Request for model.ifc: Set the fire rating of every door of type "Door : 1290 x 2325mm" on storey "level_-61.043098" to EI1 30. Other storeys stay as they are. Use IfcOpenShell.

First a look at what the model holds.

```python
import ifcopenshell
import ifcopenshell.util.element

model = ifcopenshell.open("model.ifc")
print(model.schema)
storey = next(s for s in model.by_type("IfcBuildingStorey") if s.Name == "level_-61.043098")
doors = [e for e in ifcopenshell.util.element.get_decomposition(storey) if e.is_a("IfcDoor")]
seen = {}
for e in doors:
    element_type = ifcopenshell.util.element.get_type(e)
    key = (element_type.Name if element_type != e and element_type else None, ifcopenshell.util.element.get_pset(e, "Pset_DoorCommon", "FireRating"))
    seen[key] = seen.get(key, 0) + 1
for (name, value), count in sorted(seen.items(), key=str):
    print(count, "x", name, "|", value)
```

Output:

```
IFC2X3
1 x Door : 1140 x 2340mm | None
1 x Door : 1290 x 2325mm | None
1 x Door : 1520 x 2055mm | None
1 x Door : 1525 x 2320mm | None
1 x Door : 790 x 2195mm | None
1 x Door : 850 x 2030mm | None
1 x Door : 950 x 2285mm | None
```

```python
import ifcopenshell
import ifcopenshell.api.pset
import ifcopenshell.util.element

model = ifcopenshell.open("model.ifc")

storey = next(s for s in model.by_type("IfcBuildingStorey") if s.Name == "level_-61.043098")
doors = [e for e in ifcopenshell.util.element.get_decomposition(storey) if e.is_a("IfcDoor")]

count = 0
for e in doors:
    element_type = ifcopenshell.util.element.get_type(e)
    if element_type in (None, e) or element_type.Name != "Door : 1290 x 2325mm":
        continue
    # add_pset returns the element's existing set when there is one.
    pset = ifcopenshell.api.pset.add_pset(model, product=e, name="Pset_DoorCommon")
    ifcopenshell.api.pset.edit_pset(model, pset=pset, properties={"FireRating": "EI1 30"})
    count += 1

print(count, "doors updated")

model.write("model-out.ifc")
```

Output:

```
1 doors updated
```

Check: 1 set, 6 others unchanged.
